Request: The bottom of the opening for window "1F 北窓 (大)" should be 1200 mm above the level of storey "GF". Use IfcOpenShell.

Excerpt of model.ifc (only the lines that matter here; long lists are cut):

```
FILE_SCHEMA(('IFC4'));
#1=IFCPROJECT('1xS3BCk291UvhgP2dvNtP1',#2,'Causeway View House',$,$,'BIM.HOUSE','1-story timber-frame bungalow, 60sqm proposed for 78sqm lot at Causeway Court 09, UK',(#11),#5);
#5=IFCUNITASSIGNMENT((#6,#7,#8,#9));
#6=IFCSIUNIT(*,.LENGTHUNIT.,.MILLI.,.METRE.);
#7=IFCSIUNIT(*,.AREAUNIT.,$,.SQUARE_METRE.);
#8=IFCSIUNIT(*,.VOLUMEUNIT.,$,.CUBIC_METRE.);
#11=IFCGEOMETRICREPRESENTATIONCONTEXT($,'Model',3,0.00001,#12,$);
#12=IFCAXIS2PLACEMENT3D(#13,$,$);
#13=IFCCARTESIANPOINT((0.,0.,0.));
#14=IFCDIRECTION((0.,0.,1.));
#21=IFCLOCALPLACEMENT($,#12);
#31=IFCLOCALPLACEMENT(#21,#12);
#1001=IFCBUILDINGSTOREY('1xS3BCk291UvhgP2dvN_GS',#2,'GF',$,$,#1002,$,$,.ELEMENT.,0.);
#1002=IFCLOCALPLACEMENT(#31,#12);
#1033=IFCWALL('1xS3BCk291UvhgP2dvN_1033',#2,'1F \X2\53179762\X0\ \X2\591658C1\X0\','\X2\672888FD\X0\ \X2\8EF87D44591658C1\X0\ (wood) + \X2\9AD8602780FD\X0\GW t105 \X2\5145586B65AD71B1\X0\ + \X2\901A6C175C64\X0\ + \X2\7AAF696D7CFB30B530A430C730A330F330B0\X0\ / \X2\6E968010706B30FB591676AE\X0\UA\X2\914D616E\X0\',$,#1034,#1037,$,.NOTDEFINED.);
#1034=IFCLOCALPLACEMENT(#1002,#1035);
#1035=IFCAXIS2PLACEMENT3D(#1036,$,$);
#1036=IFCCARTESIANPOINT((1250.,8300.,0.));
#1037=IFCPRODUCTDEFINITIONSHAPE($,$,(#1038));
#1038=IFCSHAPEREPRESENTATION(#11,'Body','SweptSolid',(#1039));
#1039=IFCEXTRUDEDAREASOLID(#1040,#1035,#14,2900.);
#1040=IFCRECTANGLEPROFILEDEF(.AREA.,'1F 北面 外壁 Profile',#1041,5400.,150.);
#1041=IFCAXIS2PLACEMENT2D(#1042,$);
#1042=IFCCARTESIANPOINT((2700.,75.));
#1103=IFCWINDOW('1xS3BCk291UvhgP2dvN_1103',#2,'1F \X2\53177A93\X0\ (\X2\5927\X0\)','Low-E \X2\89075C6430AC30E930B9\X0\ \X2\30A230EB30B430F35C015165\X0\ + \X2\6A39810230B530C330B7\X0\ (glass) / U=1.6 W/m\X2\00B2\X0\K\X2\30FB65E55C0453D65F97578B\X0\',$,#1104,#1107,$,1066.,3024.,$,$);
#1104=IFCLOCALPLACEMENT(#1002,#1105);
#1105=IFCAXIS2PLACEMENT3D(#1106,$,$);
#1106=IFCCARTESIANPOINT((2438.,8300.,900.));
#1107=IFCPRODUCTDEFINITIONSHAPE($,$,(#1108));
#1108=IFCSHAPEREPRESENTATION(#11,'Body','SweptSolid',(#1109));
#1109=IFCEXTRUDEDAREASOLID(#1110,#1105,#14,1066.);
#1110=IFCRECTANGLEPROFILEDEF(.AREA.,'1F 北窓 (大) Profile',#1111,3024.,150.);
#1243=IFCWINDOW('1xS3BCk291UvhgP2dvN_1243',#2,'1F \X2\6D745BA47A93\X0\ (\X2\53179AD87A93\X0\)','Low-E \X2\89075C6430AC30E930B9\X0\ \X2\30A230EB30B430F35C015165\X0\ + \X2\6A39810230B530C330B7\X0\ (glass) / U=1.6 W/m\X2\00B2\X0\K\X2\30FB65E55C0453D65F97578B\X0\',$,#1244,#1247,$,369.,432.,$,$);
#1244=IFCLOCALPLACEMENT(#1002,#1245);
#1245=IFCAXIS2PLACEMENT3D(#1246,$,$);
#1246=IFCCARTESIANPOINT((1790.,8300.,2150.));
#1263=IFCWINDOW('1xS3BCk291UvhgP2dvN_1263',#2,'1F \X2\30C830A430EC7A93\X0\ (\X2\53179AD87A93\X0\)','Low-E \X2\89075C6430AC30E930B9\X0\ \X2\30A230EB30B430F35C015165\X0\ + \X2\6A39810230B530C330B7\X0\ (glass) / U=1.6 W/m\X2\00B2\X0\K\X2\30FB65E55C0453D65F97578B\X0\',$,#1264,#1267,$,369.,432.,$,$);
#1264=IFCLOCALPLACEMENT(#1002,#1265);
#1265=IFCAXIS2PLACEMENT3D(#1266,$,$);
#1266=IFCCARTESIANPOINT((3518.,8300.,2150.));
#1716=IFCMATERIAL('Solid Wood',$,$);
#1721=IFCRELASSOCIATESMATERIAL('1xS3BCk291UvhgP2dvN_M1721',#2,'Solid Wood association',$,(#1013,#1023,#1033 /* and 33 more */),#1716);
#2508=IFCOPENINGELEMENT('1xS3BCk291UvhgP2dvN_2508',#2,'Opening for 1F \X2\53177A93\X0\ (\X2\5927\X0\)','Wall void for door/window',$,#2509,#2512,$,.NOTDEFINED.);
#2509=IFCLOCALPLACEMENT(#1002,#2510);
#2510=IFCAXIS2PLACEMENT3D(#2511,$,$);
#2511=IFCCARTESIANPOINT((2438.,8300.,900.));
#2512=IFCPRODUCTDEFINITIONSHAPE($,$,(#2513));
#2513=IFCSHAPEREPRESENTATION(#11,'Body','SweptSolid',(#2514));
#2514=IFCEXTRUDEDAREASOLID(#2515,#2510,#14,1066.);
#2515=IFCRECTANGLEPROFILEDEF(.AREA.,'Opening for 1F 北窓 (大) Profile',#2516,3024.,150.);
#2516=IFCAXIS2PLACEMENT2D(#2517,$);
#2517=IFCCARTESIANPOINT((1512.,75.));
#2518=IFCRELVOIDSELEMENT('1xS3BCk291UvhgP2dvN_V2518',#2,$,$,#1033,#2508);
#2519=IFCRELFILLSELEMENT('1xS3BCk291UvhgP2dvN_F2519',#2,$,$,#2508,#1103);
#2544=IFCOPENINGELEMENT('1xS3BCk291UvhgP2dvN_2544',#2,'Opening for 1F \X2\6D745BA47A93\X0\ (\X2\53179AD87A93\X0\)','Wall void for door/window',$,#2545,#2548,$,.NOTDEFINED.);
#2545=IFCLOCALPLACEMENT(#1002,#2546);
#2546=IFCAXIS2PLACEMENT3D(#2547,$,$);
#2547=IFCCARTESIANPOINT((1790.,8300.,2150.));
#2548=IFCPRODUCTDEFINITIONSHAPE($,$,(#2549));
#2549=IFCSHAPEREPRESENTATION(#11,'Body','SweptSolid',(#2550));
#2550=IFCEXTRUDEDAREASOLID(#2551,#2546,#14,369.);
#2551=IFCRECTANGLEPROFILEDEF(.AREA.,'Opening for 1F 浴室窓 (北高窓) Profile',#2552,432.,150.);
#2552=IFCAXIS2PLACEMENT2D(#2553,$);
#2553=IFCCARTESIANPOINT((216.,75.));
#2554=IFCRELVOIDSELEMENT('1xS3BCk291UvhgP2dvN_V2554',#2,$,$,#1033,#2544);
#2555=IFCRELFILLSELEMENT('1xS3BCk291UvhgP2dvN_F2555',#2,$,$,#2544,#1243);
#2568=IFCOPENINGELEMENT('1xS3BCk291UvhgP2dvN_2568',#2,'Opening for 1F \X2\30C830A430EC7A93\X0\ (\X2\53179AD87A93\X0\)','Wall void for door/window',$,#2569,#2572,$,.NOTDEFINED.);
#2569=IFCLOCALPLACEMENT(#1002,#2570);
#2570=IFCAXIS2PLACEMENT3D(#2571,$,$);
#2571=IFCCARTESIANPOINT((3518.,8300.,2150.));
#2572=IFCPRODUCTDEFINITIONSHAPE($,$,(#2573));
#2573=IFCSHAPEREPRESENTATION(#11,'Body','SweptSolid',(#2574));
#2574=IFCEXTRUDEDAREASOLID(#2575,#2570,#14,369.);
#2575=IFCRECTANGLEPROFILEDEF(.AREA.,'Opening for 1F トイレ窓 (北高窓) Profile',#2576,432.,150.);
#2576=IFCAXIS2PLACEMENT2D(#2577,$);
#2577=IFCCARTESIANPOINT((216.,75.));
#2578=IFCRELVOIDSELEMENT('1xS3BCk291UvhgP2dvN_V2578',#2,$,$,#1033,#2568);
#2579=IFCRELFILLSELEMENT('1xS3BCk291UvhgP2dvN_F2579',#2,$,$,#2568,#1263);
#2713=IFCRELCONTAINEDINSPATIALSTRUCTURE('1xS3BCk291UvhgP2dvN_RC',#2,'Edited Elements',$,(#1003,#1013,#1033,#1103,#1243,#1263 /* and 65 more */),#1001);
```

```python
import numpy as np
import ifcopenshell
import ifcopenshell.api.geometry
import ifcopenshell.geom
import ifcopenshell.util.element
import ifcopenshell.util.placement
import ifcopenshell.util.shape
import ifcopenshell.util.unit

model = ifcopenshell.open("model.ifc")
unit_scale = ifcopenshell.util.unit.calculate_unit_scale(model)

window = model.by_guid("1xS3BCk291UvhgP2dvN_1103")
opening = window.FillsVoids[0].RelatingOpeningElement
storey = ifcopenshell.util.element.get_container(window, ifc_class="IfcBuildingStorey")
level = ifcopenshell.util.placement.get_local_placement(storey.ObjectPlacement)[2, 3]

# The opening's origin need not be at the sill, so measure its lowest point.
shape = ifcopenshell.geom.create_shape(ifcopenshell.geom.settings(), opening)
bottom = ifcopenshell.util.shape.get_shape_bottom_elevation(shape, shape.geometry) / unit_scale
dz = level + 1200.0 - bottom

shift = np.array([0.0, 0.0, dz])
# The window is not placed relative to its opening, so move both.
for product in (opening, window):
    matrix = ifcopenshell.util.placement.get_local_placement(product.ObjectPlacement)
    matrix[:3, 3] += shift
    ifcopenshell.api.geometry.edit_object_placement(model, product=product, matrix=matrix, is_si=False)

print(f"moved by {dz * unit_scale:+.3f} m")

model.write("model_updated.ifc")
```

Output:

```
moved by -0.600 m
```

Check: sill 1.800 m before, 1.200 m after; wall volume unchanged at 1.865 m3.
